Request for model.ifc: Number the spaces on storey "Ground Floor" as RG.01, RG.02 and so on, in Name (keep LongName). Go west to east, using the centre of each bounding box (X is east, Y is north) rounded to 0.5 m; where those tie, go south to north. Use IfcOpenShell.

First a look at what the model holds.

```python
import ifcopenshell
import ifcopenshell.util.element
import ifcopenshell.util.placement

model = ifcopenshell.open("model.ifc")
print(model.schema)
storey = next(s for s in model.by_type("IfcBuildingStorey") if s.Name == "Ground Floor")
spaces = [e for e in ifcopenshell.util.element.get_decomposition(storey) if e.is_a("IfcSpace")]
for e in sorted(spaces, key=lambda e: e.id()):
    origin = ifcopenshell.util.placement.get_local_placement(e.ObjectPlacement)[:3, 3]
    print(e.id(), e.Name, e.LongName, origin.round(2) + 0.0, sep=" | ")
```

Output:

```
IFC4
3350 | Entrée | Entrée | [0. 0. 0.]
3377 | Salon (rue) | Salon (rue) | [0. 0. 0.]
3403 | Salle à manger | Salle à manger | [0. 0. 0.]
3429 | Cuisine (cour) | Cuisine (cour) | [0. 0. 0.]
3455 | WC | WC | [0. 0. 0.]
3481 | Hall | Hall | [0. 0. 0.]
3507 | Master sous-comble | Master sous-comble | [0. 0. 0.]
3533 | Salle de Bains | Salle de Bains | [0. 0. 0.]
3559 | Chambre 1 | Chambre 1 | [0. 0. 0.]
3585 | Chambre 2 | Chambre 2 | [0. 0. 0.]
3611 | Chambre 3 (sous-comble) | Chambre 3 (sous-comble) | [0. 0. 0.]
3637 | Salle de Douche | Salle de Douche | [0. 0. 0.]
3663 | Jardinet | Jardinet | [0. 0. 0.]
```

```python
import ifcopenshell
import ifcopenshell.geom
import ifcopenshell.util.element
import ifcopenshell.util.shape

model = ifcopenshell.open("model.ifc")
settings = ifcopenshell.geom.settings()
settings.set("use-world-coords", True)


def centre(element):
    shape = ifcopenshell.geom.create_shape(settings, element)
    return ifcopenshell.util.shape.get_bbox_centroid(shape.geometry)


storey = next(s for s in model.by_type("IfcBuildingStorey") if s.Name == "Ground Floor")
spaces = [e for e in ifcopenshell.util.element.get_decomposition(storey) if e.is_a("IfcSpace")]

# Insertion points can sit at a corner or the storey origin, so sort by the geometry (in metres).
centres = {e: centre(e) for e in spaces}
spaces.sort(key=lambda e: (round(centres[e][0] / 0.5), centres[e][1]))

for i, e in enumerate(spaces, start=1):
    number = f"RG.{i:02d}"
    e.Name = number
    print(e.id(), number)

model.write("model_rev.ifc")
```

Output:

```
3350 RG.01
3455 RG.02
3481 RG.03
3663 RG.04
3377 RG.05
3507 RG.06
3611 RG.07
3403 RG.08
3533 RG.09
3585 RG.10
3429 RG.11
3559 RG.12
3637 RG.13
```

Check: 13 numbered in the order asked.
